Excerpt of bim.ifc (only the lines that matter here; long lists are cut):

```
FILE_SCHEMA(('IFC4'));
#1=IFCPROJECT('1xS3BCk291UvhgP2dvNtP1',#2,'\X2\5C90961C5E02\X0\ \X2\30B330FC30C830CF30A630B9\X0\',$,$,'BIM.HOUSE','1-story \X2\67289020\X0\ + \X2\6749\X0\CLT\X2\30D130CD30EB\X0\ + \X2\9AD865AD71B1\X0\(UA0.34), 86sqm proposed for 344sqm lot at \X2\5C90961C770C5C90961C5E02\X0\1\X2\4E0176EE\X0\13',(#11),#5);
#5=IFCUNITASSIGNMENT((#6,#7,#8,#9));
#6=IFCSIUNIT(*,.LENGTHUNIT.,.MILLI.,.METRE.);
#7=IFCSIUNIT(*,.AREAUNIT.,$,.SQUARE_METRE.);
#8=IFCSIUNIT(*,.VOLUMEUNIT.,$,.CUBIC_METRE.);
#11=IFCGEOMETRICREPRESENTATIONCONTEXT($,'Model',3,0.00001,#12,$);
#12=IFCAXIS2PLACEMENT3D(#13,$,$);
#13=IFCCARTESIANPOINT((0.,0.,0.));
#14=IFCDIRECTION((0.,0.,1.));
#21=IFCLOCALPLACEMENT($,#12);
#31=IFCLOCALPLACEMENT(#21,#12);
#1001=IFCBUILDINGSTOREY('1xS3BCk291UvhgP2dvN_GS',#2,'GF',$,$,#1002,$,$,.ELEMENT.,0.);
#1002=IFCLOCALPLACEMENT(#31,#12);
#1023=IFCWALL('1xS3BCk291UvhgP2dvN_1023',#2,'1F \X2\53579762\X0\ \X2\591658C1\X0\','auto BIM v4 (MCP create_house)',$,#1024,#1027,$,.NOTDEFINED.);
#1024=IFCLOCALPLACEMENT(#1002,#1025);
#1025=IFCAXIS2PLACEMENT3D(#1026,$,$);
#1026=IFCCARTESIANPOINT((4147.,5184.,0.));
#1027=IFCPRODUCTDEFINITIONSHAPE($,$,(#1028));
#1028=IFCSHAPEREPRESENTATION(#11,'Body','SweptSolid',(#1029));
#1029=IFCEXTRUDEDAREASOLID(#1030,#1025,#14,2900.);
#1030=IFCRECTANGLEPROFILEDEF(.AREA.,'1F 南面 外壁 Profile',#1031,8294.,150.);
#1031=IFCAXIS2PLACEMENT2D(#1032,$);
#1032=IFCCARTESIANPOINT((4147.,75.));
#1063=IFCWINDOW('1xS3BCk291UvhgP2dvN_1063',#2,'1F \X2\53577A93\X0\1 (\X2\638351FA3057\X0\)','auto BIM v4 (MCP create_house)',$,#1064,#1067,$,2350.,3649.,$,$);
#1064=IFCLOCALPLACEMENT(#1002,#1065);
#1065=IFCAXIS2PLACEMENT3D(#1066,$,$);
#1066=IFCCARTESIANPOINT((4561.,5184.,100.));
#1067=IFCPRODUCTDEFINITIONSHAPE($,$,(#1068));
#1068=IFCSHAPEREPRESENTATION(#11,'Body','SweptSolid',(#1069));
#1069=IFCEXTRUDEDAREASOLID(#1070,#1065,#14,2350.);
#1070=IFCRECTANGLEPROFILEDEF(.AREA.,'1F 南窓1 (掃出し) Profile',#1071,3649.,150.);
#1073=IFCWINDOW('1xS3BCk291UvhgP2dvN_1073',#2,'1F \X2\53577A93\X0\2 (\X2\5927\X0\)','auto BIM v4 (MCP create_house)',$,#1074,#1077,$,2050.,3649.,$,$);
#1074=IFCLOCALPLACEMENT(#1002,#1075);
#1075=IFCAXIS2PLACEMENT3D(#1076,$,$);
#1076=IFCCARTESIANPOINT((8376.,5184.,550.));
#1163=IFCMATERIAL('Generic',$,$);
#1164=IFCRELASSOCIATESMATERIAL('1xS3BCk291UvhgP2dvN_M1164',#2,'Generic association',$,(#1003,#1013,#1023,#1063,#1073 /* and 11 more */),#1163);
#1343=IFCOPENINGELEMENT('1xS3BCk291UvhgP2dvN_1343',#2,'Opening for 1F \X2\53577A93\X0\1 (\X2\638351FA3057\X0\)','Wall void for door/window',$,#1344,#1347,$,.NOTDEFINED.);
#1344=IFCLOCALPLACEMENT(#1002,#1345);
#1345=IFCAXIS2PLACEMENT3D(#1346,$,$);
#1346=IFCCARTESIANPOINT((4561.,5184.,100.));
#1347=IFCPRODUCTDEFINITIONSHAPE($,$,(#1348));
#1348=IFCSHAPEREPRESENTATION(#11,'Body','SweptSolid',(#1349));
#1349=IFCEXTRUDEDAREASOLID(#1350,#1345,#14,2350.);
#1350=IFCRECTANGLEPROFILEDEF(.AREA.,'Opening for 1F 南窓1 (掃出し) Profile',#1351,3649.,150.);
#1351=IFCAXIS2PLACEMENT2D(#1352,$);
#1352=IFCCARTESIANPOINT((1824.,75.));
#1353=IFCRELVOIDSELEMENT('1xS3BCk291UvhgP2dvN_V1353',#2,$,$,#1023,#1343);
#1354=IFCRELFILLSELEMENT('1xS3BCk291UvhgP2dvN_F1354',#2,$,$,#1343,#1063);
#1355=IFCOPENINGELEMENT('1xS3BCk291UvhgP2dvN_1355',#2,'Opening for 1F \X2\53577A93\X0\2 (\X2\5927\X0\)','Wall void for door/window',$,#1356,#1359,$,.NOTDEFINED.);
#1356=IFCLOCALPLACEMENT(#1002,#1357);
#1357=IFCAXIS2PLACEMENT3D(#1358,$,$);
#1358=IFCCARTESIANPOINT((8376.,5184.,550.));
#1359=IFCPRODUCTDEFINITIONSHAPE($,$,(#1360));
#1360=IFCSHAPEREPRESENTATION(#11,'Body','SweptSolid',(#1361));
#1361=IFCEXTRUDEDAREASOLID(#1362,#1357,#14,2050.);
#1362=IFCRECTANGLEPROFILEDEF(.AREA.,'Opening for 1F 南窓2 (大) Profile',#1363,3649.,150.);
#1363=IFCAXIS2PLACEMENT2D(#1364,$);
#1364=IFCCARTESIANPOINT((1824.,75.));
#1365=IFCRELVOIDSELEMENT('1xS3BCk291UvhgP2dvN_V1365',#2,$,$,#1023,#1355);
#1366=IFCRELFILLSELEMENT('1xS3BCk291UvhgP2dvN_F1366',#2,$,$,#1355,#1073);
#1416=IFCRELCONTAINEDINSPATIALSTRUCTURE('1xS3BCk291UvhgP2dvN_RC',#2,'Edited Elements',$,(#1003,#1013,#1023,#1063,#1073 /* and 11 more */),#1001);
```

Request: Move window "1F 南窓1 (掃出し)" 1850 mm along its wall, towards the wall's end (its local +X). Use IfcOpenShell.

```python
import ifcopenshell
import ifcopenshell.api.geometry
import ifcopenshell.util.placement
import ifcopenshell.util.unit

model = ifcopenshell.open("bim.ifc")
unit_scale = ifcopenshell.util.unit.calculate_unit_scale(model)

window = model.by_guid("1xS3BCk291UvhgP2dvN_1063")
opening = window.FillsVoids[0].RelatingOpeningElement
wall = opening.VoidsElements[0].RelatingBuildingElement

wall_matrix = ifcopenshell.util.placement.get_local_placement(wall.ObjectPlacement)
shift = wall_matrix[:3, 0] * 1.85 / unit_scale
before = ifcopenshell.util.placement.get_local_placement(window.ObjectPlacement)[:3, 3].copy()

# The window is not placed relative to its opening, so move both.
for product in (opening, window):
    matrix = ifcopenshell.util.placement.get_local_placement(product.ObjectPlacement)
    matrix[:3, 3] += shift
    ifcopenshell.api.geometry.edit_object_placement(model, product=product, matrix=matrix, is_si=False)

after = ifcopenshell.util.placement.get_local_placement(window.ObjectPlacement)[:3, 3]
print("window moved by", (after - before).round(3) + 0.0)

model.write("bim_rev.ifc")
```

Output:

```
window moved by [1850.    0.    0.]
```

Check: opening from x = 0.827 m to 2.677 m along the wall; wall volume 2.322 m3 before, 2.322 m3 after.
